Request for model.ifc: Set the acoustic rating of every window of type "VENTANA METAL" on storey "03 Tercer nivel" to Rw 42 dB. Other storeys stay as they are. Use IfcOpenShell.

First a look at what the model holds.

```python
import ifcopenshell
import ifcopenshell.util.element

model = ifcopenshell.open("model.ifc")
print(model.schema)
storey = next(s for s in model.by_type("IfcBuildingStorey") if s.Name == "03 Tercer nivel")
windows = [e for e in ifcopenshell.util.element.get_decomposition(storey) if e.is_a("IfcWindow")]
seen = {}
for e in windows:
    element_type = ifcopenshell.util.element.get_type(e)
    key = (element_type.Name if element_type != e and element_type else None, ifcopenshell.util.element.get_pset(e, "Pset_WindowCommon", "AcousticRating"))
    seen[key] = seen.get(key, 0) + 1
for (name, value), count in sorted(seen.items(), key=str):
    print(count, "x", name, "|", value)
```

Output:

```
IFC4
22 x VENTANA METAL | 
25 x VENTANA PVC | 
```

```python
import ifcopenshell
import ifcopenshell.api.pset
import ifcopenshell.util.element

model = ifcopenshell.open("model.ifc")

storey = next(s for s in model.by_type("IfcBuildingStorey") if s.Name == "03 Tercer nivel")
windows = [e for e in ifcopenshell.util.element.get_decomposition(storey) if e.is_a("IfcWindow")]

count = 0
for e in windows:
    element_type = ifcopenshell.util.element.get_type(e)
    if element_type in (None, e) or element_type.Name != "VENTANA METAL":
        continue
    # add_pset returns the element's existing set when there is one.
    pset = ifcopenshell.api.pset.add_pset(model, product=e, name="Pset_WindowCommon")
    ifcopenshell.api.pset.edit_pset(model, pset=pset, properties={"AcousticRating": "Rw 42 dB"})
    count += 1

print(count, "windows updated")

model.write("model_edited.ifc")
```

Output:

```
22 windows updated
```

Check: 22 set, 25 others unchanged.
